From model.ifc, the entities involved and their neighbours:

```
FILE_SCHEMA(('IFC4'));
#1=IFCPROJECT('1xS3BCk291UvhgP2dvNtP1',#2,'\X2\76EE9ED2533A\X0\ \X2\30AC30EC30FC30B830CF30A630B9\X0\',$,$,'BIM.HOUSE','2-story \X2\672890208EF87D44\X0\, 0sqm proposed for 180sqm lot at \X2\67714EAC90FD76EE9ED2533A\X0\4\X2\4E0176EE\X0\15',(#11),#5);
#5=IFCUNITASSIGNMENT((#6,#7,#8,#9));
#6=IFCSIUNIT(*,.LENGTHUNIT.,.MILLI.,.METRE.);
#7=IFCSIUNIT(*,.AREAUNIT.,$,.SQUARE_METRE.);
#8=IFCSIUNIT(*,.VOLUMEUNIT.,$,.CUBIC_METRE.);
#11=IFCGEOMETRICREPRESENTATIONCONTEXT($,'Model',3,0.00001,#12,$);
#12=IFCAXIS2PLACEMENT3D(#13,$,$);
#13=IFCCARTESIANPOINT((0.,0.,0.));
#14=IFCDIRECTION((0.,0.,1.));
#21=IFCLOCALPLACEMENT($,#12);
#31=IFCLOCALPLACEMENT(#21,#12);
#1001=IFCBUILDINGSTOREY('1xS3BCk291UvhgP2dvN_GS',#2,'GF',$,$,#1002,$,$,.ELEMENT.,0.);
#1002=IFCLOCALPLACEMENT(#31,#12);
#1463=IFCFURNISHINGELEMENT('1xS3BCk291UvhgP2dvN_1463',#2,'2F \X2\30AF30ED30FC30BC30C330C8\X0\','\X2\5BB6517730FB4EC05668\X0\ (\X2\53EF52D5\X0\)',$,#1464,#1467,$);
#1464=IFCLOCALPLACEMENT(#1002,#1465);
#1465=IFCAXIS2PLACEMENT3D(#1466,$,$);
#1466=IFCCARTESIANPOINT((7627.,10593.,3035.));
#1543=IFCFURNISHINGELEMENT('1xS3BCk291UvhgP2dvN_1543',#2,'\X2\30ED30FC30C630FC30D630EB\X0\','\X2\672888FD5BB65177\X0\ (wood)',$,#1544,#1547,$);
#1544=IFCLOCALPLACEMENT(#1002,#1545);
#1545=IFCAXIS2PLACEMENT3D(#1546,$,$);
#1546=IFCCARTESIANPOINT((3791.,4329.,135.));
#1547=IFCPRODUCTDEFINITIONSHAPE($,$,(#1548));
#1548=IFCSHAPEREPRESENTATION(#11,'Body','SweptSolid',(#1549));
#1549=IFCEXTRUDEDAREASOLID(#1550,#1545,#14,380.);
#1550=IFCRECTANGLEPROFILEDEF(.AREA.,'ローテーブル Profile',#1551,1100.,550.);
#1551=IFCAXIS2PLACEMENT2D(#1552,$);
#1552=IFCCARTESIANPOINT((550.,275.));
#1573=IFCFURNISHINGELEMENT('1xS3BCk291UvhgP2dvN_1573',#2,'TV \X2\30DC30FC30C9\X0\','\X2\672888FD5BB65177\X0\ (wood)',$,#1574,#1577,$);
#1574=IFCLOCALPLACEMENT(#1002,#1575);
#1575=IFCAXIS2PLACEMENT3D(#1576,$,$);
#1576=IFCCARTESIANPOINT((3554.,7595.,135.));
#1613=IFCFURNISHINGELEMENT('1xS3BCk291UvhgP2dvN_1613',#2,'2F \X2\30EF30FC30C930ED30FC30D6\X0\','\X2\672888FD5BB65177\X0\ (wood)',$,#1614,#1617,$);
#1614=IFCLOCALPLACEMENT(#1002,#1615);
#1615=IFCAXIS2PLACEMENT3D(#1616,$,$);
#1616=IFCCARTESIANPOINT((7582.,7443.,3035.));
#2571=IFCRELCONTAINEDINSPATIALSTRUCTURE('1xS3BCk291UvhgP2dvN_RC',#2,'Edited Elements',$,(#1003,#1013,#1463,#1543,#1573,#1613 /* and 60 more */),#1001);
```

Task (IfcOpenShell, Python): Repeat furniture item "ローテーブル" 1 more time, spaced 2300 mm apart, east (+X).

```python
import numpy as np
import ifcopenshell
import ifcopenshell.api.geometry
import ifcopenshell.api.root
import ifcopenshell.util.element
import ifcopenshell.util.placement
import ifcopenshell.util.unit

model = ifcopenshell.open("model.ifc")
unit_scale = ifcopenshell.util.unit.calculate_unit_scale(model)


def reuse_history(source, copy):
    """copy_class also copies each property set's owner history, people and application; keep the originals."""
    for rel in copy.IsDefinedBy:
        if rel.is_a("IfcRelDefinesByProperties") and (history := rel.RelatingPropertyDefinition.OwnerHistory):
            rel.RelatingPropertyDefinition.OwnerHistory = source.OwnerHistory
            ifcopenshell.util.element.remove_deep2(model, history)


source = model.by_guid("1xS3BCk291UvhgP2dvN_1543")
base = ifcopenshell.util.placement.get_local_placement(source.ObjectPlacement)
step = np.array([1.0, 0.0, 0.0]) * 2.3 / unit_scale

for i in range(1, 2):
    copy = ifcopenshell.api.root.copy_class(model, product=source)
    copy.Representation = ifcopenshell.util.element.copy_deep(
        model, source.Representation, exclude=["IfcGeometricRepresentationContext", "IfcRepresentationMap"]
    )
    reuse_history(source, copy)
    matrix = base.copy()
    matrix[:3, 3] += i * step
    print("added at", matrix[:3, 3].round(3) + 0.0)
    ifcopenshell.api.geometry.edit_object_placement(model, product=copy, matrix=matrix, is_si=False)

model.write("model_edited.ifc")
```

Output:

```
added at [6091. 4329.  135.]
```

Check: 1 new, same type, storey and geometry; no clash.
